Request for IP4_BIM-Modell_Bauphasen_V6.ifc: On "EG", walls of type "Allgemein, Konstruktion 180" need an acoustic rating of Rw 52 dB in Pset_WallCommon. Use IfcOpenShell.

First a look at what the model holds.

```python
import ifcopenshell
import ifcopenshell.util.element

model = ifcopenshell.open("IP4_BIM-Modell_Bauphasen_V6.ifc")
print(model.schema)
storey = next(s for s in model.by_type("IfcBuildingStorey") if s.Name == "EG")
walls = [e for e in ifcopenshell.util.element.get_decomposition(storey) if e.is_a("IfcWall")]
seen = {}
for e in walls:
    element_type = ifcopenshell.util.element.get_type(e)
    key = (element_type.Name if element_type != e and element_type else None, ifcopenshell.util.element.get_pset(e, "Pset_WallCommon", "AcousticRating"))
    seen[key] = seen.get(key, 0) + 1
for (name, value), count in sorted(seen.items(), key=str):
    print(count, "x", name, "|", value)
```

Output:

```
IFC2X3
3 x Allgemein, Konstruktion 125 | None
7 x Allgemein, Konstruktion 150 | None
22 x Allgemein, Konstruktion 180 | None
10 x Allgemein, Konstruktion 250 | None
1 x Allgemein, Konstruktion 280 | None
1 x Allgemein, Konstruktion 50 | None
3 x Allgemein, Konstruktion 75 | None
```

```python
import ifcopenshell
import ifcopenshell.api.pset
import ifcopenshell.util.element

model = ifcopenshell.open("IP4_BIM-Modell_Bauphasen_V6.ifc")

storey = next(s for s in model.by_type("IfcBuildingStorey") if s.Name == "EG")
walls = [e for e in ifcopenshell.util.element.get_decomposition(storey) if e.is_a("IfcWall")]

count = 0
for e in walls:
    element_type = ifcopenshell.util.element.get_type(e)
    if element_type in (None, e) or element_type.Name != "Allgemein, Konstruktion 180":
        continue
    # add_pset returns the element's existing set when there is one.
    pset = ifcopenshell.api.pset.add_pset(model, product=e, name="Pset_WallCommon")
    ifcopenshell.api.pset.edit_pset(model, pset=pset, properties={"AcousticRating": "Rw 52 dB"})
    count += 1

print(count, "walls updated")

model.write("IP4_BIM-Modell_Bauphasen_V6_updated.ifc")
```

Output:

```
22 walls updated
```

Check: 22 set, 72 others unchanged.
